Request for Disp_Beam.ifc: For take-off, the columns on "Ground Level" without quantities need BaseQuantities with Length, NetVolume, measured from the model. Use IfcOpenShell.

First a look at what the model holds.

```python
import ifcopenshell
import ifcopenshell.util.element
import ifcopenshell.util.unit

model = ifcopenshell.open("Disp_Beam.ifc")
print(model.schema)
for unit_type in ("LENGTHUNIT", "AREAUNIT", "VOLUMEUNIT"):
    print(unit_type, ifcopenshell.util.unit.calculate_unit_scale(model, unit_type))
storey = next(s for s in model.by_type("IfcBuildingStorey") if s.Name == "Ground Level")
columns = [e for e in ifcopenshell.util.element.get_decomposition(storey) if e.is_a("IfcColumn")]
for e in sorted(columns, key=lambda e: e.id()):
    print(e.id(), e.is_a(), e.Name, list(ifcopenshell.util.element.get_psets(e, qtos_only=True)), sep=" | ")
```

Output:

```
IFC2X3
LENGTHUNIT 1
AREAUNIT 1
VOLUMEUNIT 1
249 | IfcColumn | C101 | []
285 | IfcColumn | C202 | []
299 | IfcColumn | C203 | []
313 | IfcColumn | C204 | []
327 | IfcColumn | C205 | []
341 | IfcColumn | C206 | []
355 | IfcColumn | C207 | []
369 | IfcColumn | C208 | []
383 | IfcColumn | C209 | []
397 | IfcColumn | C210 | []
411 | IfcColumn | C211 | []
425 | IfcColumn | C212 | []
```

```python
import ifcopenshell
import ifcopenshell.api.pset
import ifcopenshell.geom
import ifcopenshell.util.element
import ifcopenshell.util.shape
import ifcopenshell.util.unit

model = ifcopenshell.open("Disp_Beam.ifc")
unit_scale = ifcopenshell.util.unit.calculate_unit_scale(model)
volume_scale = ifcopenshell.util.unit.calculate_unit_scale(model, "VOLUMEUNIT")
settings = ifcopenshell.geom.settings()

storey = next(s for s in model.by_type("IfcBuildingStorey") if s.Name == "Ground Level")
columns = [e for e in ifcopenshell.util.element.get_decomposition(storey) if e.is_a("IfcColumn")]

for e in sorted(columns, key=lambda e: e.id()):
    if ifcopenshell.util.element.get_psets(e, qtos_only=True, should_inherit=False):
        continue
    # Geometry comes back in metres, in the element's own axes.
    shape = ifcopenshell.geom.create_shape(settings, e)
    values = {
        "Length": ifcopenshell.util.shape.get_z(shape.geometry) / unit_scale,
        "NetVolume": ifcopenshell.util.shape.get_volume(shape.geometry) / volume_scale,
    }
    qto = ifcopenshell.api.pset.add_qto(model, product=e, name="BaseQuantities")
    ifcopenshell.api.pset.edit_qto(model, qto=qto, properties=values)
    print(e.id(), {k: round(v, 3) for k, v in values.items()})

model.write("Disp_Beam_rev.ifc")
```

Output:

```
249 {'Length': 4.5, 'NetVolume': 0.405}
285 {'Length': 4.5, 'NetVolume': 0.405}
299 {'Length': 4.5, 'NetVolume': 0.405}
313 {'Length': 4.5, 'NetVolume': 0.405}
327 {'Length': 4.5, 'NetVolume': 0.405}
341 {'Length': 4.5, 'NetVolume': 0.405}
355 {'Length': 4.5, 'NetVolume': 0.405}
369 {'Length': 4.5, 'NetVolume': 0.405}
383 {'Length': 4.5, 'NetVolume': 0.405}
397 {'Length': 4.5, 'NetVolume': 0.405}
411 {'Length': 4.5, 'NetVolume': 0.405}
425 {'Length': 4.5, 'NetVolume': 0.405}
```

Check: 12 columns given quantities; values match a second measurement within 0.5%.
